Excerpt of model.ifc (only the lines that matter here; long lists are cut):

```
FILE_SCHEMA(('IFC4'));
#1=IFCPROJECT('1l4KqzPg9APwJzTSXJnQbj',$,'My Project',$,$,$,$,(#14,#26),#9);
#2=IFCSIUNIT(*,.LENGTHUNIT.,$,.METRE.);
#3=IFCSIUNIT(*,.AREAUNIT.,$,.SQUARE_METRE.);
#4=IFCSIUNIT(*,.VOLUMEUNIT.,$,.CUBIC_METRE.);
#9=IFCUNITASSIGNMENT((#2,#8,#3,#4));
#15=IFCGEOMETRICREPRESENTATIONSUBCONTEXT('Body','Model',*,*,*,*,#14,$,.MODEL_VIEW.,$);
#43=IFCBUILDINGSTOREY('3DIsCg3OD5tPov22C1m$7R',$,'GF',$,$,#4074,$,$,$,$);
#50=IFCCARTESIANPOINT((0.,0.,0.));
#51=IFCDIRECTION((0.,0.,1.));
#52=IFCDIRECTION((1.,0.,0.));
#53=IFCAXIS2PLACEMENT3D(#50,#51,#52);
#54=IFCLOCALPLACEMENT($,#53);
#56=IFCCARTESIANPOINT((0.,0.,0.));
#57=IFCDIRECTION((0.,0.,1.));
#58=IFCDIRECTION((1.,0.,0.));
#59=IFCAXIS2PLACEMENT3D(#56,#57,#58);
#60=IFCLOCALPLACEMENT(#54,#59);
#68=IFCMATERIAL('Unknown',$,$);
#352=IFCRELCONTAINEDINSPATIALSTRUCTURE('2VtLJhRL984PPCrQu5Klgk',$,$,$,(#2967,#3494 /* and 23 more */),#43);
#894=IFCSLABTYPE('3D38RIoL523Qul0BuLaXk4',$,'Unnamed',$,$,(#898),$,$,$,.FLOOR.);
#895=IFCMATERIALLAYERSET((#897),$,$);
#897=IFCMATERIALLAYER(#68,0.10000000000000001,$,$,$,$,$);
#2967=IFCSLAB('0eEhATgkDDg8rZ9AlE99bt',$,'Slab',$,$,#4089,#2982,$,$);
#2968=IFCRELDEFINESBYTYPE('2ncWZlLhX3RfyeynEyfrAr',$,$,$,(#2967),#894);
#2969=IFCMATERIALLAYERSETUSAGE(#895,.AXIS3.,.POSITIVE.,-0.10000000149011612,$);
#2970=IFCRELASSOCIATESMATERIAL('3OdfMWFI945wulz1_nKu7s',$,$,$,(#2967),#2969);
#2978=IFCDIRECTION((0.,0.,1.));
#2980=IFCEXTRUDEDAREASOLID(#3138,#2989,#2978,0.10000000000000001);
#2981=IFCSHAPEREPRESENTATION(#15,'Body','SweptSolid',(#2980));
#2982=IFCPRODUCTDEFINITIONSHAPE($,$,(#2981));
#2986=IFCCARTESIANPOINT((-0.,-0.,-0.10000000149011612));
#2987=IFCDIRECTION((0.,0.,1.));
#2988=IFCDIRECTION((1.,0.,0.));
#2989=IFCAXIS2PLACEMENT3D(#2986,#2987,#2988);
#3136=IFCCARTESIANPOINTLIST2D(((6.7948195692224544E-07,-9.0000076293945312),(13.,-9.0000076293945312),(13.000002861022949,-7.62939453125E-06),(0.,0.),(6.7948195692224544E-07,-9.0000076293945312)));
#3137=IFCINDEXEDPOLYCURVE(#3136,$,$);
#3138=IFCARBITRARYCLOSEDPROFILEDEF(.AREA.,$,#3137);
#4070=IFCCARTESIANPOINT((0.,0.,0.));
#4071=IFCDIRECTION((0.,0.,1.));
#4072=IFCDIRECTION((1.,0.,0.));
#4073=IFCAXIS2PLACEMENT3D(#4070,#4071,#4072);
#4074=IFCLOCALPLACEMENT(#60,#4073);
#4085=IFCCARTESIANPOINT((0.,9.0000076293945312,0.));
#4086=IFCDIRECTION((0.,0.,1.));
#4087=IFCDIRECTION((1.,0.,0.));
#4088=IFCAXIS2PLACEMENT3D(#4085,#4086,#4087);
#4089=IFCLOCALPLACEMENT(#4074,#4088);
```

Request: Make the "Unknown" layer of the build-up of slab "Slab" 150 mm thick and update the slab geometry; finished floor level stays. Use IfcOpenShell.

```python
import ifcopenshell
import ifcopenshell.util.element
import ifcopenshell.util.representation

model = ifcopenshell.open("model.ifc")

layer_set = model.by_id(895)
layer = next(l for l in layer_set.MaterialLayers if l.Material and l.Material.Name == "Unknown")
change = 0.15 - layer.LayerThickness
layer.LayerThickness += change

# Geometry does not follow the layer set by itself.
slabs = [e for e in ifcopenshell.util.element.get_elements_by_material(model, layer_set) if e.is_a("IfcSlab")]
for slab in sorted(slabs, key=lambda e: e.id()):
    body = ifcopenshell.util.representation.get_representation(slab, "Model", "Body")
    solid = body.Items[0]
    old_depth = solid.Depth
    solid.Depth += change
    # Extruded upwards: lower the start of the extrusion so the top stays.
    x, y, z = solid.Position.Location.Coordinates
    solid.Position.Location = model.createIfcCartesianPoint((x, y, z - change))
    print(slab.id(), f"{old_depth:g} -> {solid.Depth:g}")

# The layers are counted up from the underside, which has moved.
for usage in {ifcopenshell.util.element.get_material(slab) for slab in slabs}:
    usage.OffsetFromReferenceLine -= change

model.write("model_updated.ifc")
```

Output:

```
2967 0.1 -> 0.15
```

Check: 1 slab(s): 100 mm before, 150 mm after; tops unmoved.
